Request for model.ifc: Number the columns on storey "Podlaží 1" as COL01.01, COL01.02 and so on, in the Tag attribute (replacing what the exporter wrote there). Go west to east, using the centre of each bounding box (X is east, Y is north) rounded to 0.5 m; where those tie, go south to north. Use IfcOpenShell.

First a look at what the model holds.

```python
import ifcopenshell
import ifcopenshell.util.element
import ifcopenshell.util.placement

model = ifcopenshell.open("model.ifc")
print(model.schema)
storey = next(s for s in model.by_type("IfcBuildingStorey") if s.Name == "Podlaží 1")
columns = [e for e in ifcopenshell.util.element.get_decomposition(storey) if e.is_a("IfcColumn")]
for e in sorted(columns, key=lambda e: e.id()):
    origin = ifcopenshell.util.placement.get_local_placement(e.ObjectPlacement)[:3, 3]
    print(e.id(), e.Tag, e.Name, origin.round(2) + 0.0, sep=" | ")
```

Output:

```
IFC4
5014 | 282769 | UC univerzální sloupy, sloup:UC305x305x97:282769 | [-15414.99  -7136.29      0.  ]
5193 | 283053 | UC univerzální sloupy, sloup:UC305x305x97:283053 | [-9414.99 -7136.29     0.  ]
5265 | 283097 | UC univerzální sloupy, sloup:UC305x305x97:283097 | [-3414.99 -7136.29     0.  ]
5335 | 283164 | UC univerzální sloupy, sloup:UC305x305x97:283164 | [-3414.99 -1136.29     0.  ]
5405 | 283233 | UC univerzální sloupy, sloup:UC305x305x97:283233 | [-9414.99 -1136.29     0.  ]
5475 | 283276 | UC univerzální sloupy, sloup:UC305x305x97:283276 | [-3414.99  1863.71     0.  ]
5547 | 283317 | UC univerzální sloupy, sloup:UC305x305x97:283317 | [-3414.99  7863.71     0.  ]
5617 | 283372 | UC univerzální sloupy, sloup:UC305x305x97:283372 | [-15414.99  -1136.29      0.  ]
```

```python
import ifcopenshell
import ifcopenshell.geom
import ifcopenshell.util.element
import ifcopenshell.util.shape

model = ifcopenshell.open("model.ifc")
settings = ifcopenshell.geom.settings()
settings.set("use-world-coords", True)


def centre(element):
    shape = ifcopenshell.geom.create_shape(settings, element)
    return ifcopenshell.util.shape.get_bbox_centroid(shape.geometry)


storey = next(s for s in model.by_type("IfcBuildingStorey") if s.Name == "Podlaží 1")
columns = [e for e in ifcopenshell.util.element.get_decomposition(storey) if e.is_a("IfcColumn")]

# Insertion points can sit at a corner or the storey origin, so sort by the geometry (in metres).
centres = {e: centre(e) for e in columns}
columns.sort(key=lambda e: (round(centres[e][0] / 0.5), centres[e][1]))

for i, e in enumerate(columns, start=1):
    number = f"COL01.{i:02d}"
    e.Tag = number
    print(e.id(), number)

model.write("model_rev.ifc")
```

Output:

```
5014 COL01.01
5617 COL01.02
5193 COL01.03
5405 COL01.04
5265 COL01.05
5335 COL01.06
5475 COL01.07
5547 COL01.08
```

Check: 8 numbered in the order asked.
